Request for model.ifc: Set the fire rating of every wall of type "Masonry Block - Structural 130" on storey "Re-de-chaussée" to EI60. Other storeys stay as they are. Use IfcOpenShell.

First a look at what the model holds.

```python
import ifcopenshell
import ifcopenshell.util.element

model = ifcopenshell.open("model.ifc")
print(model.schema)
storey = next(s for s in model.by_type("IfcBuildingStorey") if s.Name == "Re-de-chaussée")
walls = [e for e in ifcopenshell.util.element.get_decomposition(storey) if e.is_a("IfcWall")]
seen = {}
for e in walls:
    element_type = ifcopenshell.util.element.get_type(e)
    key = (element_type.Name if element_type != e and element_type else None, ifcopenshell.util.element.get_pset(e, "Pset_WallCommon", "FireRating"))
    seen[key] = seen.get(key, 0) + 1
for (name, value), count in sorted(seen.items(), key=str):
    print(count, "x", name, "|", value)
```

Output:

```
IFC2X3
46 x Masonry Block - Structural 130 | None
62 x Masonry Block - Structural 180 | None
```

```python
import ifcopenshell
import ifcopenshell.api.pset
import ifcopenshell.util.element

model = ifcopenshell.open("model.ifc")

storey = next(s for s in model.by_type("IfcBuildingStorey") if s.Name == "Re-de-chaussée")
walls = [e for e in ifcopenshell.util.element.get_decomposition(storey) if e.is_a("IfcWall")]

count = 0
for e in walls:
    element_type = ifcopenshell.util.element.get_type(e)
    if element_type in (None, e) or element_type.Name != "Masonry Block - Structural 130":
        continue
    # add_pset returns the element's existing set when there is one.
    pset = ifcopenshell.api.pset.add_pset(model, product=e, name="Pset_WallCommon")
    ifcopenshell.api.pset.edit_pset(model, pset=pset, properties={"FireRating": "EI60"})
    count += 1

print(count, "walls updated")

model.write("model-out.ifc")
```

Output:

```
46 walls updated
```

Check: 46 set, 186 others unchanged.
